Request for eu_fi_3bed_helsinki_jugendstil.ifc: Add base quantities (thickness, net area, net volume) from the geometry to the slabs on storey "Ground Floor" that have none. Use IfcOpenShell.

First a look at what the model holds.

```python
import ifcopenshell
import ifcopenshell.util.element
import ifcopenshell.util.unit

model = ifcopenshell.open("eu_fi_3bed_helsinki_jugendstil.ifc")
print(model.schema)
for unit_type in ("LENGTHUNIT", "AREAUNIT", "VOLUMEUNIT"):
    print(unit_type, ifcopenshell.util.unit.calculate_unit_scale(model, unit_type))
storey = next(s for s in model.by_type("IfcBuildingStorey") if s.Name == "Ground Floor")
slabs = [e for e in ifcopenshell.util.element.get_decomposition(storey) if e.is_a("IfcSlab")]
for e in sorted(slabs, key=lambda e: e.id()):
    print(e.id(), e.is_a(), e.Name, list(ifcopenshell.util.element.get_psets(e, qtos_only=True)), sep=" | ")
```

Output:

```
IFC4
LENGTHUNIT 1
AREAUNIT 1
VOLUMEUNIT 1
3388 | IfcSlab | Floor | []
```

```python
import ifcopenshell
import ifcopenshell.api.pset
import ifcopenshell.geom
import ifcopenshell.util.element
import ifcopenshell.util.shape
import ifcopenshell.util.unit

model = ifcopenshell.open("eu_fi_3bed_helsinki_jugendstil.ifc")
unit_scale = ifcopenshell.util.unit.calculate_unit_scale(model)
area_scale = ifcopenshell.util.unit.calculate_unit_scale(model, "AREAUNIT")
volume_scale = ifcopenshell.util.unit.calculate_unit_scale(model, "VOLUMEUNIT")
settings = ifcopenshell.geom.settings()

storey = next(s for s in model.by_type("IfcBuildingStorey") if s.Name == "Ground Floor")
slabs = [e for e in ifcopenshell.util.element.get_decomposition(storey) if e.is_a("IfcSlab")]

for e in sorted(slabs, key=lambda e: e.id()):
    if ifcopenshell.util.element.get_psets(e, qtos_only=True, should_inherit=False):
        continue
    # Geometry comes back in metres, in the element's own axes.
    shape = ifcopenshell.geom.create_shape(settings, e)
    values = {
        "Width": ifcopenshell.util.shape.get_z(shape.geometry) / unit_scale,
        "NetArea": ifcopenshell.util.shape.get_footprint_area(shape.geometry) / area_scale,
        "NetVolume": ifcopenshell.util.shape.get_volume(shape.geometry) / volume_scale,
    }
    qto = ifcopenshell.api.pset.add_qto(model, product=e, name="Qto_SlabBaseQuantities")
    ifcopenshell.api.pset.edit_qto(model, qto=qto, properties=values)
    print(e.id(), {k: round(v, 3) for k, v in values.items()})

model.write("eu_fi_3bed_helsinki_jugendstil_rev.ifc")
```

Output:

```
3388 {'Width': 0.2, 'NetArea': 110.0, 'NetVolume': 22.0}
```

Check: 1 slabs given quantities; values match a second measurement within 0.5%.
